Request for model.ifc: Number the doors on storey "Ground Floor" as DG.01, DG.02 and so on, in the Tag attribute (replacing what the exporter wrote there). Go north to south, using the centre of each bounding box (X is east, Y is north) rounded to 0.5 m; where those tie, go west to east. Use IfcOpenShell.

First a look at what the model holds.

```python
import ifcopenshell
import ifcopenshell.util.element
import ifcopenshell.util.placement

model = ifcopenshell.open("model.ifc")
print(model.schema)
storey = next(s for s in model.by_type("IfcBuildingStorey") if s.Name == "Ground Floor")
doors = [e for e in ifcopenshell.util.element.get_decomposition(storey) if e.is_a("IfcDoor")]
for e in sorted(doors, key=lambda e: e.id()):
    origin = ifcopenshell.util.placement.get_local_placement(e.ObjectPlacement)[:3, 3]
    print(e.id(), e.Tag, e.Name, origin.round(2) + 0.0, sep=" | ")
```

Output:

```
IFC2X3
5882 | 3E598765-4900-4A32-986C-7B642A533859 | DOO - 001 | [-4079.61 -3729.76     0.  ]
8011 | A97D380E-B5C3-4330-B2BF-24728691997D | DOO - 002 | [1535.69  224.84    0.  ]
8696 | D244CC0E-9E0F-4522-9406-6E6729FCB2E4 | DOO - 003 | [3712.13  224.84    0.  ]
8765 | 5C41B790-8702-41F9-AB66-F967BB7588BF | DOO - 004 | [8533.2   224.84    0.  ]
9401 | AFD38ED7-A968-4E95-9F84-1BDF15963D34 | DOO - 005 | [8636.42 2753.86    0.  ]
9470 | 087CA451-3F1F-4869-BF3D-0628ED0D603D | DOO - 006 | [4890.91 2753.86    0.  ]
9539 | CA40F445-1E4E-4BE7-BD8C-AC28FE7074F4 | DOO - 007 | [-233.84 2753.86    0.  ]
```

```python
import ifcopenshell
import ifcopenshell.geom
import ifcopenshell.util.element
import ifcopenshell.util.shape

model = ifcopenshell.open("model.ifc")
settings = ifcopenshell.geom.settings()
settings.set("use-world-coords", True)


def centre(element):
    shape = ifcopenshell.geom.create_shape(settings, element)
    return ifcopenshell.util.shape.get_bbox_centroid(shape.geometry)


storey = next(s for s in model.by_type("IfcBuildingStorey") if s.Name == "Ground Floor")
doors = [e for e in ifcopenshell.util.element.get_decomposition(storey) if e.is_a("IfcDoor")]

# Insertion points can sit at a corner or the storey origin, so sort by the geometry (in metres).
centres = {e: centre(e) for e in doors}
doors.sort(key=lambda e: (-round(centres[e][1] / 0.5), centres[e][0]))

for i, e in enumerate(doors, start=1):
    number = f"DG.{i:02d}"
    e.Tag = number
    print(e.id(), number)

model.write("model_updated.ifc")
```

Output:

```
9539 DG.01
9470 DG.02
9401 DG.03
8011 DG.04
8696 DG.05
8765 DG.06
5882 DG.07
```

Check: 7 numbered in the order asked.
